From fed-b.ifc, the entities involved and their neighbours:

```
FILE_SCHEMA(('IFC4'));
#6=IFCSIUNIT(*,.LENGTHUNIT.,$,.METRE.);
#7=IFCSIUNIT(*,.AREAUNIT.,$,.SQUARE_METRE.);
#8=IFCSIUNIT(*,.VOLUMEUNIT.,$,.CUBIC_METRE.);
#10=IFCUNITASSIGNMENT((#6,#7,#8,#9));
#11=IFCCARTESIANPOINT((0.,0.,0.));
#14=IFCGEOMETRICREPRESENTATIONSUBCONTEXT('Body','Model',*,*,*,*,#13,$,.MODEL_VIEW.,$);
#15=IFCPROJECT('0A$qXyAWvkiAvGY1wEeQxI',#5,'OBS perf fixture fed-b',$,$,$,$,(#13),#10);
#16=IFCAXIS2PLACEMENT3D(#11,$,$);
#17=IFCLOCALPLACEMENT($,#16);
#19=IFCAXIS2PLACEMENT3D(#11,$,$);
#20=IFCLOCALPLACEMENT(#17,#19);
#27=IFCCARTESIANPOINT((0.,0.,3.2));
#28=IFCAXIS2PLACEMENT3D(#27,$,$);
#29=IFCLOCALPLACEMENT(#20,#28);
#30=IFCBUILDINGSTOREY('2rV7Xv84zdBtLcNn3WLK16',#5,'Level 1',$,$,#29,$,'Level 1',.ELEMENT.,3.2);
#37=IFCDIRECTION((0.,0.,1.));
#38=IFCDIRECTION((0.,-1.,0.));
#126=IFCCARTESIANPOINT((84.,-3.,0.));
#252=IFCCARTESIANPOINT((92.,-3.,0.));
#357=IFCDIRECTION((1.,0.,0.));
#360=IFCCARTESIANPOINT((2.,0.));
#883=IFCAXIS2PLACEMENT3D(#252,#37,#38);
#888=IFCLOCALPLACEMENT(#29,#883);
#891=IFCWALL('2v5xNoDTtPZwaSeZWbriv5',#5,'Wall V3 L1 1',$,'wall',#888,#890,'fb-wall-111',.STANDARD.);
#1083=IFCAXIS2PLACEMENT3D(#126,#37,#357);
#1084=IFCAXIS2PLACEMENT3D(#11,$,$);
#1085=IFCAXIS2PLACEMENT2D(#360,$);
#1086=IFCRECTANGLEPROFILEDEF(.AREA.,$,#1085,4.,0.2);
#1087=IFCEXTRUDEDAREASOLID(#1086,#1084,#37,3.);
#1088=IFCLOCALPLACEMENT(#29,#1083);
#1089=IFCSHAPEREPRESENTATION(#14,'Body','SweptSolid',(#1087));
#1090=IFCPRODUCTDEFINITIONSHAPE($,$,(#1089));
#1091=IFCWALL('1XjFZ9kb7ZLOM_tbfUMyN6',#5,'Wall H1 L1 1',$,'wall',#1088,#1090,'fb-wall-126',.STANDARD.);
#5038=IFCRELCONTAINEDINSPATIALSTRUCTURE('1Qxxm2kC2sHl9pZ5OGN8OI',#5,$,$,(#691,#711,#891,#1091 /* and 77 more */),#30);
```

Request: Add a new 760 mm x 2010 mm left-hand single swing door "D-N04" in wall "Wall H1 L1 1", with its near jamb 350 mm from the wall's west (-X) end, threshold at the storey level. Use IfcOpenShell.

```python
import numpy as np
import ifcopenshell
import ifcopenshell.api.feature
import ifcopenshell.api.geometry
import ifcopenshell.api.root
import ifcopenshell.api.spatial
import ifcopenshell.geom
import ifcopenshell.util.element
import ifcopenshell.util.placement
import ifcopenshell.util.representation
import ifcopenshell.util.shape
import ifcopenshell.util.unit

model = ifcopenshell.open("fed-b.ifc")
unit_scale = ifcopenshell.util.unit.calculate_unit_scale(model)
settings = ifcopenshell.geom.settings()


def volume(element):
    """Net volume in cubic metres, openings subtracted."""
    shape = ifcopenshell.geom.create_shape(settings, element)
    return ifcopenshell.util.shape.get_volume(shape.geometry)


wall = model.by_guid("1XjFZ9kb7ZLOM_tbfUMyN6")
storey = ifcopenshell.util.element.get_container(wall, ifc_class="IfcBuildingStorey")
context = ifcopenshell.util.representation.get_context(model, "Model", "Body", "MODEL_VIEW")
before = volume(wall)

width, height, from_end, sill = 0.76, 2.01, 0.35, 0.0  # metres

# The wall runs along its own X axis, and the end named is its -X end.
wall_shape = ifcopenshell.geom.create_shape(settings, wall)
x, y, z = ifcopenshell.util.shape.get_vertices(wall_shape.geometry).T
start = x.min() + from_end
face, thickness = float(y.min()), float(y.max() - y.min())
wall_matrix = ifcopenshell.util.placement.get_local_placement(wall.ObjectPlacement)
level = ifcopenshell.util.placement.get_local_placement(storey.ObjectPlacement)[2, 3]


def in_wall(x, y):
    """Placement at x, y metres in the wall's axes, at sill height."""
    matrix = wall_matrix.copy()
    matrix[:, 3] = wall_matrix @ np.array([x / unit_scale, y / unit_scale, 0.0, 1.0])
    matrix[2, 3] = level + sill / unit_scale
    return matrix


# Opening: a box that overshoots both wall faces by 50 mm.
opening = ifcopenshell.api.root.create_entity(model, ifc_class="IfcOpeningElement", predefined_type="OPENING")
box = ifcopenshell.api.geometry.add_wall_representation(
    model, context=context, length=width, height=height, thickness=thickness + 0.1
)
ifcopenshell.api.geometry.assign_representation(model, product=opening, representation=box)
ifcopenshell.api.geometry.edit_object_placement(model, product=opening, matrix=in_wall(start, face - 0.05), is_si=False)
ifcopenshell.api.feature.add_feature(model, feature=opening, element=wall)

door = ifcopenshell.api.root.create_entity(model, ifc_class="IfcDoor", name="D-N04", predefined_type="DOOR")
door.OverallWidth, door.OverallHeight = width / unit_scale, height / unit_scale
door.OperationType = "SINGLE_SWING_LEFT"
body = ifcopenshell.api.geometry.add_door_representation(
    model,
    context=context,
    overall_width=door.OverallWidth,
    overall_height=door.OverallHeight,
    operation_type="SINGLE_SWING_LEFT",
    lining_properties={"LiningDepth": thickness / unit_scale, "ThresholdDepth": thickness / unit_scale},
)
ifcopenshell.api.geometry.assign_representation(model, product=door, representation=body)
ifcopenshell.api.spatial.assign_container(model, products=[door], relating_structure=storey)
ifcopenshell.api.feature.add_filling(model, opening=opening, element=door)

# The lining spans the wall, so the door starts at the wall face.
ifcopenshell.api.geometry.edit_object_placement(model, product=door, matrix=in_wall(start, face), is_si=False)

after = volume(wall)

print(f"wall volume {before:.3f} -> {after:.3f} m3")

model.write("fed-b_edited.ifc")
```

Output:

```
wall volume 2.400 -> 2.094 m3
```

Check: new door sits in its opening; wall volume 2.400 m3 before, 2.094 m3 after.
